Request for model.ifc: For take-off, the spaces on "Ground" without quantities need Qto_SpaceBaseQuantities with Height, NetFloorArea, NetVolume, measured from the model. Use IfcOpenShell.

First a look at what the model holds.

```python
import ifcopenshell
import ifcopenshell.util.element
import ifcopenshell.util.unit

model = ifcopenshell.open("model.ifc")
print(model.schema)
for unit_type in ("LENGTHUNIT", "AREAUNIT", "VOLUMEUNIT"):
    print(unit_type, ifcopenshell.util.unit.calculate_unit_scale(model, unit_type))
storey = next(s for s in model.by_type("IfcBuildingStorey") if s.Name == "Ground")
spaces = [e for e in ifcopenshell.util.element.get_decomposition(storey) if e.is_a("IfcSpace")]
for e in sorted(spaces, key=lambda e: e.id()):
    print(e.id(), e.is_a(), e.Name, list(ifcopenshell.util.element.get_psets(e, qtos_only=True)), sep=" | ")
```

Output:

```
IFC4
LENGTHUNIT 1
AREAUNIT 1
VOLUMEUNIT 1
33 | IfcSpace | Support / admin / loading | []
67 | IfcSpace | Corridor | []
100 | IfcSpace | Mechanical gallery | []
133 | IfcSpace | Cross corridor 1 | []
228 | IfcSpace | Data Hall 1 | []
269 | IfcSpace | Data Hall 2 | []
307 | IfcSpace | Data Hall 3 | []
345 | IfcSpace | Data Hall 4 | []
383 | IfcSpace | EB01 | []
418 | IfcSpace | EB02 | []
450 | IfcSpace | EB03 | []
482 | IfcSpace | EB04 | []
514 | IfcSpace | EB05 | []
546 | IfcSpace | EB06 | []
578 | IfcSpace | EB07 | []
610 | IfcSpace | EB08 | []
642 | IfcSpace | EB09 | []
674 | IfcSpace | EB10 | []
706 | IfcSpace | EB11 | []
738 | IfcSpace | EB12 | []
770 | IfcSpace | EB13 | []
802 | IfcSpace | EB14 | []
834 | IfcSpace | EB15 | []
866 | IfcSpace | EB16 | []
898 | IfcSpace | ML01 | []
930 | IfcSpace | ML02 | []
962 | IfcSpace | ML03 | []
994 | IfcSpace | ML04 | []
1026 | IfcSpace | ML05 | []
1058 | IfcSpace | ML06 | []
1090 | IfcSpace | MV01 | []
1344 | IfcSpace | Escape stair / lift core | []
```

```python
import ifcopenshell
import ifcopenshell.api.pset
import ifcopenshell.geom
import ifcopenshell.util.element
import ifcopenshell.util.shape
import ifcopenshell.util.unit

model = ifcopenshell.open("model.ifc")
unit_scale = ifcopenshell.util.unit.calculate_unit_scale(model)
area_scale = ifcopenshell.util.unit.calculate_unit_scale(model, "AREAUNIT")
volume_scale = ifcopenshell.util.unit.calculate_unit_scale(model, "VOLUMEUNIT")
settings = ifcopenshell.geom.settings()

storey = next(s for s in model.by_type("IfcBuildingStorey") if s.Name == "Ground")
spaces = [e for e in ifcopenshell.util.element.get_decomposition(storey) if e.is_a("IfcSpace")]

for e in sorted(spaces, key=lambda e: e.id()):
    if ifcopenshell.util.element.get_psets(e, qtos_only=True, should_inherit=False):
        continue
    # Geometry comes back in metres, in the element's own axes.
    shape = ifcopenshell.geom.create_shape(settings, e)
    values = {
        "Height": ifcopenshell.util.shape.get_z(shape.geometry) / unit_scale,
        "NetFloorArea": ifcopenshell.util.shape.get_footprint_area(shape.geometry) / area_scale,
        "NetVolume": ifcopenshell.util.shape.get_volume(shape.geometry) / volume_scale,
    }
    qto = ifcopenshell.api.pset.add_qto(model, product=e, name="Qto_SpaceBaseQuantities")
    ifcopenshell.api.pset.edit_qto(model, qto=qto, properties=values)
    print(e.id(), {k: round(v, 3) for k, v in values.items()})

model.write("model_rev.ifc")
```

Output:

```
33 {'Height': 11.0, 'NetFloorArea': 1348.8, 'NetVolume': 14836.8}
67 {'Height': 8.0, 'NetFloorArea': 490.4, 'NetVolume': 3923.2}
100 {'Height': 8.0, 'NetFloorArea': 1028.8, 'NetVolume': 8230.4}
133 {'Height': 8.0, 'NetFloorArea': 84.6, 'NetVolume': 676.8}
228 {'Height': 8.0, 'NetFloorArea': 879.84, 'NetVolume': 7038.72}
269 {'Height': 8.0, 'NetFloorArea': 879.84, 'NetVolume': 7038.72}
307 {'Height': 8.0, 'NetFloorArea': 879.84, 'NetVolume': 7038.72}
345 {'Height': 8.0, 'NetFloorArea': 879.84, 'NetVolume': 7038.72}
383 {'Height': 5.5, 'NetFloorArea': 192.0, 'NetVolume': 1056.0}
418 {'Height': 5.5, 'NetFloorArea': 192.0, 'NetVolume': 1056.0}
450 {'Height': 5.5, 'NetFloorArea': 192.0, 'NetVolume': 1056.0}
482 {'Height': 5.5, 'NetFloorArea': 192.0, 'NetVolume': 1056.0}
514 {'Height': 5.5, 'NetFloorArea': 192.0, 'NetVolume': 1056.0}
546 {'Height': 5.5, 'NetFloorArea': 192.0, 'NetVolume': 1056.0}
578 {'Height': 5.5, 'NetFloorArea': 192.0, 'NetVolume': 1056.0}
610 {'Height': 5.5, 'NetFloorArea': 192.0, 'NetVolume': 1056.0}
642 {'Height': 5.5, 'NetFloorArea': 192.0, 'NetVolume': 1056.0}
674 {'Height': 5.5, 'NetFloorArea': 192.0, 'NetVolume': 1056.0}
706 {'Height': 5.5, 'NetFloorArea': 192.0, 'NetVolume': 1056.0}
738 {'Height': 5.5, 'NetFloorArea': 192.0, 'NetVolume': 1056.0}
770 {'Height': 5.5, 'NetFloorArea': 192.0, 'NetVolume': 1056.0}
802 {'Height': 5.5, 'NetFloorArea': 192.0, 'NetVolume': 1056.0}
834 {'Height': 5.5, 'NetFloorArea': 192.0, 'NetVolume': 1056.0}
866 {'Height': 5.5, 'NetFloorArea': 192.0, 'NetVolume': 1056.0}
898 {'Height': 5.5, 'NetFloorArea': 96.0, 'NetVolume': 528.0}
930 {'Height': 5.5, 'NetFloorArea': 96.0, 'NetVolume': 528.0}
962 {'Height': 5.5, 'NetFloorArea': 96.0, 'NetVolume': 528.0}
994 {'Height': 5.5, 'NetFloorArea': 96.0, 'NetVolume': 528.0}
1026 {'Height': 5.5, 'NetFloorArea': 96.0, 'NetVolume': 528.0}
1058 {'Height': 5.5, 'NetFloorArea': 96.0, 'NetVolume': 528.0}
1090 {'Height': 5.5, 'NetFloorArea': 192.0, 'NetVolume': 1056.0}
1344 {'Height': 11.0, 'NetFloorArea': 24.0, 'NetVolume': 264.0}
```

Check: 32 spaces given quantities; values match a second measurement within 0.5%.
